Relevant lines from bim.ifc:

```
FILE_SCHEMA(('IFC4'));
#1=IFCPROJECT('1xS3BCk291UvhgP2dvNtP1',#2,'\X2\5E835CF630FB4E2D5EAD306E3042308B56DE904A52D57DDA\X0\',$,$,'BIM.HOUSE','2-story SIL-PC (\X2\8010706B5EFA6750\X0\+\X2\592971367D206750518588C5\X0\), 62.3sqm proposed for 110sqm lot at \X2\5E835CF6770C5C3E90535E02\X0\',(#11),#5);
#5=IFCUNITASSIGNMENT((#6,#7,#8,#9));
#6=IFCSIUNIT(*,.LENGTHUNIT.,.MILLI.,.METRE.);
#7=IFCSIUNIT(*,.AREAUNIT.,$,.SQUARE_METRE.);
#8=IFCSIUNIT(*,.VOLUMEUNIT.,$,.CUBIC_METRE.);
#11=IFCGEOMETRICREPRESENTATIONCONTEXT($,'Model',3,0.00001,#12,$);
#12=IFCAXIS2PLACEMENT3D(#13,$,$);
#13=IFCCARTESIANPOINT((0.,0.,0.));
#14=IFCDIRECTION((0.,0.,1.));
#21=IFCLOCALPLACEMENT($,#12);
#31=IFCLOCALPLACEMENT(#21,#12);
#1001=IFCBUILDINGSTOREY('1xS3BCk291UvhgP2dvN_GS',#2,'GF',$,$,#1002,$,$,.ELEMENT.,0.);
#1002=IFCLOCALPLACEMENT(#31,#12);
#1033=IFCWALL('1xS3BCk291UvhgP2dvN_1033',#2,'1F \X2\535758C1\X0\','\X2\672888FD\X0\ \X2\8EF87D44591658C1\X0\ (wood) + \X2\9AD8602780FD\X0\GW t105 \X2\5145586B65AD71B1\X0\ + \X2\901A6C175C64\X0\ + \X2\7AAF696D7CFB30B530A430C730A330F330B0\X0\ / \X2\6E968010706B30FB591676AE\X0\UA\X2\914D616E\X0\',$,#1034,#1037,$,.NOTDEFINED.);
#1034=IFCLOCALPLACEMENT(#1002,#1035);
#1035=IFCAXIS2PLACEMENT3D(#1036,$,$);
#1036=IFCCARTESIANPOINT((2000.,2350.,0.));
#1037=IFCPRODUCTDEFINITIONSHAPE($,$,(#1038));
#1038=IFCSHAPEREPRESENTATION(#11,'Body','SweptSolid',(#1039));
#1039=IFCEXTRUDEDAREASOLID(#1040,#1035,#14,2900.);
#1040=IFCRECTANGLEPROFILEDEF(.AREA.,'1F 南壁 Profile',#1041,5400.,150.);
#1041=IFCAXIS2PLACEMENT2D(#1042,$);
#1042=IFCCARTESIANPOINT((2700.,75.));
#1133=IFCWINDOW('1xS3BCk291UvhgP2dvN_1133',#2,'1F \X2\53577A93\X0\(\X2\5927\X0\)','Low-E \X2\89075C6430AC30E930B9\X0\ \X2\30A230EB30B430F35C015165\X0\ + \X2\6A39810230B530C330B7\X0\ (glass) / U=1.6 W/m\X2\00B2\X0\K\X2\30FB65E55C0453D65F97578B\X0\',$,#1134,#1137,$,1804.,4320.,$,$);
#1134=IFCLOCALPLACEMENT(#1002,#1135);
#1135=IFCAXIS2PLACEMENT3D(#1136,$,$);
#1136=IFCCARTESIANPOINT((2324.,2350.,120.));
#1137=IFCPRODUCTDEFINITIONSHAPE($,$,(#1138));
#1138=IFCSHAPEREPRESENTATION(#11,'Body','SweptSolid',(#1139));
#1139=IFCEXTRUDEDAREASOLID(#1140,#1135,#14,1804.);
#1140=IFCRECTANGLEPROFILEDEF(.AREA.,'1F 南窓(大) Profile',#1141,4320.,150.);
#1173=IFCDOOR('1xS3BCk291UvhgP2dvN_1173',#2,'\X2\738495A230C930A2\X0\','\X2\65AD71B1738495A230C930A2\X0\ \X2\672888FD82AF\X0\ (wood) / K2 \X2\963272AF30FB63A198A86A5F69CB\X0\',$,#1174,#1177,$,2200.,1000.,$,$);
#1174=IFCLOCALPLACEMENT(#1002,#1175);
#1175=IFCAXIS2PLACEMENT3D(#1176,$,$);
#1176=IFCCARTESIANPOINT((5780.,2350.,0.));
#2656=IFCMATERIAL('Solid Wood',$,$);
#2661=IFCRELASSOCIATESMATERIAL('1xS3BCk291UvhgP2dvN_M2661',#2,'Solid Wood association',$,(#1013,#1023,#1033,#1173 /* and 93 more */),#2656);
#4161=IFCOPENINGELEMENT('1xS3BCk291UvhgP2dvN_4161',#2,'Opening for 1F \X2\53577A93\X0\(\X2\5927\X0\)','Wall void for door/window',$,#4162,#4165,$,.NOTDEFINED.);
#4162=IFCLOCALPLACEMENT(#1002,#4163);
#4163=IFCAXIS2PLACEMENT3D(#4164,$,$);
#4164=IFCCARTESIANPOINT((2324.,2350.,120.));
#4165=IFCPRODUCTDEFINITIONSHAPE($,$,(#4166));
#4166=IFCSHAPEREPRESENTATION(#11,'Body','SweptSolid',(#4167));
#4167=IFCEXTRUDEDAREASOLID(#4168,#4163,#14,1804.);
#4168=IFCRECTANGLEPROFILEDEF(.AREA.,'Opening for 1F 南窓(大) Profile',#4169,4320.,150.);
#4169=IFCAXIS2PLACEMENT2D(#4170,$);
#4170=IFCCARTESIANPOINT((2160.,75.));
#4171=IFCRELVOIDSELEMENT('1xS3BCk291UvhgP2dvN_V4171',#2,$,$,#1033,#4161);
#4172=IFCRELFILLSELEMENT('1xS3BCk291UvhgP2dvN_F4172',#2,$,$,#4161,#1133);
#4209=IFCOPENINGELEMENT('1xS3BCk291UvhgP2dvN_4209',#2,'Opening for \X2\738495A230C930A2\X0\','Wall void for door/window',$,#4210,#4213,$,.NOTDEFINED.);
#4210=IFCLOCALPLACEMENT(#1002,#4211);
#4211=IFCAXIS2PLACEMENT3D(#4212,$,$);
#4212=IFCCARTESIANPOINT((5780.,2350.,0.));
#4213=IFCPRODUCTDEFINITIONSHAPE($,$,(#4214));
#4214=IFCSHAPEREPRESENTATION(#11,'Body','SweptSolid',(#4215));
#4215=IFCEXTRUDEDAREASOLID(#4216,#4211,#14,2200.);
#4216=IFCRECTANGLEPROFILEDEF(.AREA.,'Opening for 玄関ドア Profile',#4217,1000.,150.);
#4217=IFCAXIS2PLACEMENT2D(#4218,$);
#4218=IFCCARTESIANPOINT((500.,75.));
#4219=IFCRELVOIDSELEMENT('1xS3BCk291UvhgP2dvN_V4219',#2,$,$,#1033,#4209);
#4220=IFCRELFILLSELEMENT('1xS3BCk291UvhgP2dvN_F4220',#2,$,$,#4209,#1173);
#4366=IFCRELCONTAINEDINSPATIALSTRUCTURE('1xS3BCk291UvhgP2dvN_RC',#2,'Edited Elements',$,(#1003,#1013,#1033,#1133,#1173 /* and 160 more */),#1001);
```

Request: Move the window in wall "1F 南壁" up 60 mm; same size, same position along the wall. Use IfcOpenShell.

```python
import numpy as np
import ifcopenshell
import ifcopenshell.api.geometry
import ifcopenshell.util.placement
import ifcopenshell.util.unit

model = ifcopenshell.open("bim.ifc")
unit_scale = ifcopenshell.util.unit.calculate_unit_scale(model)

window = model.by_guid("1xS3BCk291UvhgP2dvN_1133")
opening = window.FillsVoids[0].RelatingOpeningElement
dz = 0.06 / unit_scale

shift = np.array([0.0, 0.0, dz])
# The window is not placed relative to its opening, so move both.
for product in (opening, window):
    matrix = ifcopenshell.util.placement.get_local_placement(product.ObjectPlacement)
    matrix[:3, 3] += shift
    ifcopenshell.api.geometry.edit_object_placement(model, product=product, matrix=matrix, is_si=False)

print(f"moved by {dz * unit_scale:+.3f} m")

model.write("bim_rev.ifc")
```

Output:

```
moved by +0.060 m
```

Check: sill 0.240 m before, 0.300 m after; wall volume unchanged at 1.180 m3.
